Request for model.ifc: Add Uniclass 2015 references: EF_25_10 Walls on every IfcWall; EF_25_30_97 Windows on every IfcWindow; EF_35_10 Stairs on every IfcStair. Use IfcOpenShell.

First a look at what the model holds.

```python
import ifcopenshell

model = ifcopenshell.open("model.ifc")
print(model.schema)
print("classifications:", [c.Name for c in model.by_type("IfcClassification")])
for ifc_class in ("IfcDoor", "IfcRoof", "IfcStair", "IfcWall", "IfcWindow"):
    print(ifc_class, len(model.by_type(ifc_class)))
```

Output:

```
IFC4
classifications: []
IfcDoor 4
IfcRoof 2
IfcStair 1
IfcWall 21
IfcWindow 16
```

```python
import ifcopenshell
import ifcopenshell.api.classification

model = ifcopenshell.open("model.ifc")

system = ifcopenshell.api.classification.add_classification(model, classification="Uniclass 2015")

codes = {
    "IfcWall": ("EF_25_10", "Walls"),
    "IfcWindow": ("EF_25_30_97", "Windows"),
    "IfcStair": ("EF_35_10", "Stairs"),
}
for ifc_class, (code, name) in codes.items():
    products = model.by_type(ifc_class)
    ifcopenshell.api.classification.add_reference(
        model, products=products, classification=system, identification=code, name=name
    )
    print(code, len(products))

model.write("model_rev.ifc")
```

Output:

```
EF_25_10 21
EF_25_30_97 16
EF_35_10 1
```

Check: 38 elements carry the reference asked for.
